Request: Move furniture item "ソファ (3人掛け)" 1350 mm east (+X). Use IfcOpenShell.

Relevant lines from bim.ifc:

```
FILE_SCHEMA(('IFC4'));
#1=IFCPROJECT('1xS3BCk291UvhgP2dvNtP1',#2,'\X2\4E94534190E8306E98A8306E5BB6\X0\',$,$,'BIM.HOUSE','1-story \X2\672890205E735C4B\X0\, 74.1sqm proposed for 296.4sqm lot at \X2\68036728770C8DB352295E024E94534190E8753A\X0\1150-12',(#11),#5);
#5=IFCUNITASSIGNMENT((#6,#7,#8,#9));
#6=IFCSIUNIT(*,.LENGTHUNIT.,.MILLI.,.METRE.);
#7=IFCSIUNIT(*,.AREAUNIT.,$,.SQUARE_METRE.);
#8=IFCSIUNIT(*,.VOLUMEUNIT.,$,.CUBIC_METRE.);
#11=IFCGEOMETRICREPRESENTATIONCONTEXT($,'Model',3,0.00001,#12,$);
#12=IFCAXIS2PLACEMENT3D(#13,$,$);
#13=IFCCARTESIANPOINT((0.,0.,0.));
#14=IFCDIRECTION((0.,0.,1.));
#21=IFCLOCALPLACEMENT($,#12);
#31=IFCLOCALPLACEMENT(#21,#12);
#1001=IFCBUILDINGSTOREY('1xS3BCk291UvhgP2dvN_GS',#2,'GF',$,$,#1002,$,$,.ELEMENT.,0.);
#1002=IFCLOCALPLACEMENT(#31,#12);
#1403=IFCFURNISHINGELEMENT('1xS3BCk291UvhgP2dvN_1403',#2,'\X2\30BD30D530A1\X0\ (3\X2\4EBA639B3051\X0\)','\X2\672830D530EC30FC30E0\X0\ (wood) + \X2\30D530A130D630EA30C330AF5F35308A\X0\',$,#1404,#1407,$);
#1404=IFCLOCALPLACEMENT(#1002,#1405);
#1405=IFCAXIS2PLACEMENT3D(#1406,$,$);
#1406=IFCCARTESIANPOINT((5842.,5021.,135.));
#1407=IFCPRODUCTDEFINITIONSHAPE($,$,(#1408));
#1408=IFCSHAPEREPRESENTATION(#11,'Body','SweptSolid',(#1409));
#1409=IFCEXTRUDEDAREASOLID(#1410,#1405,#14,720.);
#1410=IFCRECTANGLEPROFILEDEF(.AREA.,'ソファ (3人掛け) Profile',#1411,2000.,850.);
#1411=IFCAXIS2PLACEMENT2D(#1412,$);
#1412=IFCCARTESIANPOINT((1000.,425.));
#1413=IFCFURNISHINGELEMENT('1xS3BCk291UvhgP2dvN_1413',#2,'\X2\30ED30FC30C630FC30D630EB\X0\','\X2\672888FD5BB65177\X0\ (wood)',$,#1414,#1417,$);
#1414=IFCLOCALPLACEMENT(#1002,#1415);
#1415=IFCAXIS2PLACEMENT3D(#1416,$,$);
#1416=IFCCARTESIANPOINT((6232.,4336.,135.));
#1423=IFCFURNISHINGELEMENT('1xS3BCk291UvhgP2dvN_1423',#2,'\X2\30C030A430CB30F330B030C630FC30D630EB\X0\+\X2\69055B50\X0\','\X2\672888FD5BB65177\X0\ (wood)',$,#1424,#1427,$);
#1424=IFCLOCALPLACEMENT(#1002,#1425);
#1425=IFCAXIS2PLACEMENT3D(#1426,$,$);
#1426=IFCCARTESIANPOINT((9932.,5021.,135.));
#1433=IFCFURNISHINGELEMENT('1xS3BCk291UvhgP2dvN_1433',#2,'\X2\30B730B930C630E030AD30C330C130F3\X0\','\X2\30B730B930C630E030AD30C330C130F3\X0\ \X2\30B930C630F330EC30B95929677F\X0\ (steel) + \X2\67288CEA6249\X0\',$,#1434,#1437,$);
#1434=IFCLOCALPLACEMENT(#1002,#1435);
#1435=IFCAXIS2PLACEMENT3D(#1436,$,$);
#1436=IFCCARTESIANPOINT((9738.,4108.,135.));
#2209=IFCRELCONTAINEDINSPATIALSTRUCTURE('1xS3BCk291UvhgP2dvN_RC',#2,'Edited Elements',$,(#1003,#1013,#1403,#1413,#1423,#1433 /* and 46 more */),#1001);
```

```python
import ifcopenshell
import ifcopenshell.api.geometry
import ifcopenshell.util.placement
import ifcopenshell.util.unit

model = ifcopenshell.open("bim.ifc")
unit_scale = ifcopenshell.util.unit.calculate_unit_scale(model)

item = model.by_guid("1xS3BCk291UvhgP2dvN_1403")
matrix = ifcopenshell.util.placement.get_local_placement(item.ObjectPlacement)
matrix[0, 3] += 1.35 / unit_scale
ifcopenshell.api.geometry.edit_object_placement(model, product=item, matrix=matrix, is_si=False)

print(ifcopenshell.util.placement.get_local_placement(item.ObjectPlacement).round(3) + 0.0)

model.write("bim-out.ifc")
```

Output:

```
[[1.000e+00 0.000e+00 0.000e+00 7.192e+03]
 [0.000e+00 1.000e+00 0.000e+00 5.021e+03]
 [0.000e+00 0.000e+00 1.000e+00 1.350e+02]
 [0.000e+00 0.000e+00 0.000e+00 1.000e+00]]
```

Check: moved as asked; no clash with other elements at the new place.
